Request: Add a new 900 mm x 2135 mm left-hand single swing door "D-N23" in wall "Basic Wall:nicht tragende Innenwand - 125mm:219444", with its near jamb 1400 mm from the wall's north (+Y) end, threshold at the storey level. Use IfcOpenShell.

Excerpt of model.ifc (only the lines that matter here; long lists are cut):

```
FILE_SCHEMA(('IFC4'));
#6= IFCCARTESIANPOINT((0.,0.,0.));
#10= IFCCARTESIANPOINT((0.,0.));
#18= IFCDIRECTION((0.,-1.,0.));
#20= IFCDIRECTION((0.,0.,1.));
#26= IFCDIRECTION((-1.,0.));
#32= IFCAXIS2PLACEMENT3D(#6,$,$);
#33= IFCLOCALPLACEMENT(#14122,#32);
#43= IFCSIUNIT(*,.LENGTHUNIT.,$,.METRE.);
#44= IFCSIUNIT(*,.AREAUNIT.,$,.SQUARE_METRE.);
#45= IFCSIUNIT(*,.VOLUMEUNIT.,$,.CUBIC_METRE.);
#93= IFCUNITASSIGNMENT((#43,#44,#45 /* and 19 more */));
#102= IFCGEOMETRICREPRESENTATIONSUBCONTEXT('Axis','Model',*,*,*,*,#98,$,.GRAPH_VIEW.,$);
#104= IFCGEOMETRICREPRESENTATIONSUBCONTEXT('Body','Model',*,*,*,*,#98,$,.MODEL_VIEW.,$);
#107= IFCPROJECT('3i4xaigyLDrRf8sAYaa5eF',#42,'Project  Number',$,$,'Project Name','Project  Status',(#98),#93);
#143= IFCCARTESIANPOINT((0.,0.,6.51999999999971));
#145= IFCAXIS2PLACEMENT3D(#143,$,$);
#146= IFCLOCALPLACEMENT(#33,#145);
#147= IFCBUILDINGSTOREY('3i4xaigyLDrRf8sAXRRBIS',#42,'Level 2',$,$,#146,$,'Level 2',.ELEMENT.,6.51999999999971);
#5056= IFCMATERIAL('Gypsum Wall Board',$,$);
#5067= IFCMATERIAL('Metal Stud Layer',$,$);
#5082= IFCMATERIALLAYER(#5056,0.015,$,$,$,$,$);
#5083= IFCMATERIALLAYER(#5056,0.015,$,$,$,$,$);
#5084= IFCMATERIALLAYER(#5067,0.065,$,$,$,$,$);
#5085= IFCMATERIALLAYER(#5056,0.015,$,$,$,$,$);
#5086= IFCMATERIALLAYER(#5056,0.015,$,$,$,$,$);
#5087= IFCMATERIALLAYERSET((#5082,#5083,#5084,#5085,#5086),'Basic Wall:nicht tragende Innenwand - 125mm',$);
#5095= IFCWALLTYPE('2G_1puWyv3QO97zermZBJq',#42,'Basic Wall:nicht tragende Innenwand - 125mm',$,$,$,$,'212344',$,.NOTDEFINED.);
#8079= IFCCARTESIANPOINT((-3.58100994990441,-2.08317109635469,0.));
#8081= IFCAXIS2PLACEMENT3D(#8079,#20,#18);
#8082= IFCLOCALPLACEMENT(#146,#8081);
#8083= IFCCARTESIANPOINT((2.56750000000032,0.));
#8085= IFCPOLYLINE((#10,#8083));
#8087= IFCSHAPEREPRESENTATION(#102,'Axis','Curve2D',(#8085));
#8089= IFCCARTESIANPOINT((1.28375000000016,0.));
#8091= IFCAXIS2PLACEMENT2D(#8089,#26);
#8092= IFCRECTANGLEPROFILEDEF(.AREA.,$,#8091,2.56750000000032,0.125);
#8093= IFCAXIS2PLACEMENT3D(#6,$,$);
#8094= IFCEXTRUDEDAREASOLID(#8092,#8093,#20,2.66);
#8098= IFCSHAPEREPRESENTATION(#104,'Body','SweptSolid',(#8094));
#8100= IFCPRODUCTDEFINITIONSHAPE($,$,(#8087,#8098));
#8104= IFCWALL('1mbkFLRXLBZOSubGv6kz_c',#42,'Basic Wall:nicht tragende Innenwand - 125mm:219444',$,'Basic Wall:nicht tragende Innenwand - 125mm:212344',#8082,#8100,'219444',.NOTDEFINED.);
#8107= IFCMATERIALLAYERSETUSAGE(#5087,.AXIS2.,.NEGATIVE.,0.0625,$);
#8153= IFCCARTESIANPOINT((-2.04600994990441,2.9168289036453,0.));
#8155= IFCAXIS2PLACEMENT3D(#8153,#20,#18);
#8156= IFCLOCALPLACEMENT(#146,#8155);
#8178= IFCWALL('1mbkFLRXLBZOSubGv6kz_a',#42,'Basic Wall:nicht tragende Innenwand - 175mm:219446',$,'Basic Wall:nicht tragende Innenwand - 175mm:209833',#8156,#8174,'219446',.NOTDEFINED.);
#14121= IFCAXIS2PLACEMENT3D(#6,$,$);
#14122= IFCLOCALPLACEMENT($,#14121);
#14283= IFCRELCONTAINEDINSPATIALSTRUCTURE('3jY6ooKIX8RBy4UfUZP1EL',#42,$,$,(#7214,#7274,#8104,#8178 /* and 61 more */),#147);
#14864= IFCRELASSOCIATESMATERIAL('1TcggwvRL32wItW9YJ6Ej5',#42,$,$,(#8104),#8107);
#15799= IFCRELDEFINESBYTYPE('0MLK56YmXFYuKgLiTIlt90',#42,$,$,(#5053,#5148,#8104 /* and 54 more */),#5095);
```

```python
import numpy as np
import ifcopenshell
import ifcopenshell.api.feature
import ifcopenshell.api.geometry
import ifcopenshell.api.root
import ifcopenshell.api.spatial
import ifcopenshell.geom
import ifcopenshell.util.element
import ifcopenshell.util.placement
import ifcopenshell.util.representation
import ifcopenshell.util.shape
import ifcopenshell.util.unit

model = ifcopenshell.open("model.ifc")
unit_scale = ifcopenshell.util.unit.calculate_unit_scale(model)
settings = ifcopenshell.geom.settings()


def volume(element):
    """Net volume in cubic metres, openings subtracted."""
    shape = ifcopenshell.geom.create_shape(settings, element)
    return ifcopenshell.util.shape.get_volume(shape.geometry)


wall = model.by_guid("1mbkFLRXLBZOSubGv6kz_c")
storey = ifcopenshell.util.element.get_container(wall, ifc_class="IfcBuildingStorey")
context = ifcopenshell.util.representation.get_context(model, "Model", "Body", "MODEL_VIEW")
before = volume(wall)

width, height, from_end, sill = 0.9, 2.135, 1.4, 0.0  # metres

# The wall runs along its own X axis, and the end named is its -X end.
wall_shape = ifcopenshell.geom.create_shape(settings, wall)
x, y, z = ifcopenshell.util.shape.get_vertices(wall_shape.geometry).T
start = x.min() + from_end
face, thickness = float(y.min()), float(y.max() - y.min())
wall_matrix = ifcopenshell.util.placement.get_local_placement(wall.ObjectPlacement)
level = ifcopenshell.util.placement.get_local_placement(storey.ObjectPlacement)[2, 3]


def in_wall(x, y):
    """Placement at x, y metres in the wall's axes, at sill height."""
    matrix = wall_matrix.copy()
    matrix[:, 3] = wall_matrix @ np.array([x / unit_scale, y / unit_scale, 0.0, 1.0])
    matrix[2, 3] = level + sill / unit_scale
    return matrix


# Opening: a box that overshoots both wall faces by 50 mm.
opening = ifcopenshell.api.root.create_entity(model, ifc_class="IfcOpeningElement", predefined_type="OPENING")
box = ifcopenshell.api.geometry.add_wall_representation(
    model, context=context, length=width, height=height, thickness=thickness + 0.1
)
ifcopenshell.api.geometry.assign_representation(model, product=opening, representation=box)
ifcopenshell.api.geometry.edit_object_placement(model, product=opening, matrix=in_wall(start, face - 0.05), is_si=False)
ifcopenshell.api.feature.add_feature(model, feature=opening, element=wall)

door = ifcopenshell.api.root.create_entity(model, ifc_class="IfcDoor", name="D-N23", predefined_type="DOOR")
door.OverallWidth, door.OverallHeight = width / unit_scale, height / unit_scale
door.OperationType = "SINGLE_SWING_LEFT"
body = ifcopenshell.api.geometry.add_door_representation(
    model,
    context=context,
    overall_width=door.OverallWidth,
    overall_height=door.OverallHeight,
    operation_type="SINGLE_SWING_LEFT",
    lining_properties={"LiningDepth": thickness / unit_scale, "ThresholdDepth": thickness / unit_scale},
)
ifcopenshell.api.geometry.assign_representation(model, product=door, representation=body)
ifcopenshell.api.spatial.assign_container(model, products=[door], relating_structure=storey)
ifcopenshell.api.feature.add_filling(model, opening=opening, element=door)

# The lining spans the wall, so the door starts at the wall face.
ifcopenshell.api.geometry.edit_object_placement(model, product=door, matrix=in_wall(start, face), is_si=False)

after = volume(wall)

print(f"wall volume {before:.3f} -> {after:.3f} m3")

model.write("model_updated.ifc")
```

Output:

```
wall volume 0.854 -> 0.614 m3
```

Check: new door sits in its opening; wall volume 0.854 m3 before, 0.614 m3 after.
